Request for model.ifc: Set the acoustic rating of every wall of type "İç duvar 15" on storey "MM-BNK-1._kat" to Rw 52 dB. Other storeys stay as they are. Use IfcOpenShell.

First a look at what the model holds.

```python
import ifcopenshell
import ifcopenshell.util.element

model = ifcopenshell.open("model.ifc")
print(model.schema)
storey = next(s for s in model.by_type("IfcBuildingStorey") if s.Name == "MM-BNK-1._kat")
walls = [e for e in ifcopenshell.util.element.get_decomposition(storey) if e.is_a("IfcWall")]
seen = {}
for e in walls:
    element_type = ifcopenshell.util.element.get_type(e)
    key = (element_type.Name if element_type != e and element_type else None, ifcopenshell.util.element.get_pset(e, "Pset_WallCommon", "AcousticRating"))
    seen[key] = seen.get(key, 0) + 1
for (name, value), count in sorted(seen.items(), key=str):
    print(count, "x", name, "|", value)
```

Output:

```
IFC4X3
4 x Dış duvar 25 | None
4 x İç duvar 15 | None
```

```python
import ifcopenshell
import ifcopenshell.api.pset
import ifcopenshell.util.element

model = ifcopenshell.open("model.ifc")

storey = next(s for s in model.by_type("IfcBuildingStorey") if s.Name == "MM-BNK-1._kat")
walls = [e for e in ifcopenshell.util.element.get_decomposition(storey) if e.is_a("IfcWall")]

count = 0
for e in walls:
    element_type = ifcopenshell.util.element.get_type(e)
    if element_type in (None, e) or element_type.Name != "İç duvar 15":
        continue
    # add_pset returns the element's existing set when there is one.
    pset = ifcopenshell.api.pset.add_pset(model, product=e, name="Pset_WallCommon")
    ifcopenshell.api.pset.edit_pset(model, pset=pset, properties={"AcousticRating": "Rw 52 dB"})
    count += 1

print(count, "walls updated")

model.write("model_edited.ifc")
```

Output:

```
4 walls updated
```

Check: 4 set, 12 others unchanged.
